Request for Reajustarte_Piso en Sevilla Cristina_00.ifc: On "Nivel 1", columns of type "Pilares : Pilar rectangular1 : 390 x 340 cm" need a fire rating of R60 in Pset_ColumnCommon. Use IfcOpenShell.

First a look at what the model holds.

```python
import ifcopenshell
import ifcopenshell.util.element

model = ifcopenshell.open("Reajustarte_Piso en Sevilla Cristina_00.ifc")
print(model.schema)
storey = next(s for s in model.by_type("IfcBuildingStorey") if s.Name == "Nivel 1")
columns = [e for e in ifcopenshell.util.element.get_decomposition(storey) if e.is_a("IfcColumn")]
seen = {}
for e in columns:
    element_type = ifcopenshell.util.element.get_type(e)
    key = (element_type.Name if element_type != e and element_type else None, ifcopenshell.util.element.get_pset(e, "Pset_ColumnCommon", "FireRating"))
    seen[key] = seen.get(key, 0) + 1
for (name, value), count in sorted(seen.items(), key=str):
    print(count, "x", name, "|", value)
```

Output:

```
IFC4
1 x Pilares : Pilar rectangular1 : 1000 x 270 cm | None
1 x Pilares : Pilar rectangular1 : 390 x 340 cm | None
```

```python
import ifcopenshell
import ifcopenshell.api.pset
import ifcopenshell.util.element

model = ifcopenshell.open("Reajustarte_Piso en Sevilla Cristina_00.ifc")

storey = next(s for s in model.by_type("IfcBuildingStorey") if s.Name == "Nivel 1")
columns = [e for e in ifcopenshell.util.element.get_decomposition(storey) if e.is_a("IfcColumn")]

count = 0
for e in columns:
    element_type = ifcopenshell.util.element.get_type(e)
    if element_type in (None, e) or element_type.Name != "Pilares : Pilar rectangular1 : 390 x 340 cm":
        continue
    # add_pset returns the element's existing set when there is one.
    pset = ifcopenshell.api.pset.add_pset(model, product=e, name="Pset_ColumnCommon")
    ifcopenshell.api.pset.edit_pset(model, pset=pset, properties={"FireRating": "R60"})
    count += 1

print(count, "columns updated")

model.write("Reajustarte_Piso en Sevilla Cristina_00_v2.ifc")
```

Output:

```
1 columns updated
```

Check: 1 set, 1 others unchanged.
